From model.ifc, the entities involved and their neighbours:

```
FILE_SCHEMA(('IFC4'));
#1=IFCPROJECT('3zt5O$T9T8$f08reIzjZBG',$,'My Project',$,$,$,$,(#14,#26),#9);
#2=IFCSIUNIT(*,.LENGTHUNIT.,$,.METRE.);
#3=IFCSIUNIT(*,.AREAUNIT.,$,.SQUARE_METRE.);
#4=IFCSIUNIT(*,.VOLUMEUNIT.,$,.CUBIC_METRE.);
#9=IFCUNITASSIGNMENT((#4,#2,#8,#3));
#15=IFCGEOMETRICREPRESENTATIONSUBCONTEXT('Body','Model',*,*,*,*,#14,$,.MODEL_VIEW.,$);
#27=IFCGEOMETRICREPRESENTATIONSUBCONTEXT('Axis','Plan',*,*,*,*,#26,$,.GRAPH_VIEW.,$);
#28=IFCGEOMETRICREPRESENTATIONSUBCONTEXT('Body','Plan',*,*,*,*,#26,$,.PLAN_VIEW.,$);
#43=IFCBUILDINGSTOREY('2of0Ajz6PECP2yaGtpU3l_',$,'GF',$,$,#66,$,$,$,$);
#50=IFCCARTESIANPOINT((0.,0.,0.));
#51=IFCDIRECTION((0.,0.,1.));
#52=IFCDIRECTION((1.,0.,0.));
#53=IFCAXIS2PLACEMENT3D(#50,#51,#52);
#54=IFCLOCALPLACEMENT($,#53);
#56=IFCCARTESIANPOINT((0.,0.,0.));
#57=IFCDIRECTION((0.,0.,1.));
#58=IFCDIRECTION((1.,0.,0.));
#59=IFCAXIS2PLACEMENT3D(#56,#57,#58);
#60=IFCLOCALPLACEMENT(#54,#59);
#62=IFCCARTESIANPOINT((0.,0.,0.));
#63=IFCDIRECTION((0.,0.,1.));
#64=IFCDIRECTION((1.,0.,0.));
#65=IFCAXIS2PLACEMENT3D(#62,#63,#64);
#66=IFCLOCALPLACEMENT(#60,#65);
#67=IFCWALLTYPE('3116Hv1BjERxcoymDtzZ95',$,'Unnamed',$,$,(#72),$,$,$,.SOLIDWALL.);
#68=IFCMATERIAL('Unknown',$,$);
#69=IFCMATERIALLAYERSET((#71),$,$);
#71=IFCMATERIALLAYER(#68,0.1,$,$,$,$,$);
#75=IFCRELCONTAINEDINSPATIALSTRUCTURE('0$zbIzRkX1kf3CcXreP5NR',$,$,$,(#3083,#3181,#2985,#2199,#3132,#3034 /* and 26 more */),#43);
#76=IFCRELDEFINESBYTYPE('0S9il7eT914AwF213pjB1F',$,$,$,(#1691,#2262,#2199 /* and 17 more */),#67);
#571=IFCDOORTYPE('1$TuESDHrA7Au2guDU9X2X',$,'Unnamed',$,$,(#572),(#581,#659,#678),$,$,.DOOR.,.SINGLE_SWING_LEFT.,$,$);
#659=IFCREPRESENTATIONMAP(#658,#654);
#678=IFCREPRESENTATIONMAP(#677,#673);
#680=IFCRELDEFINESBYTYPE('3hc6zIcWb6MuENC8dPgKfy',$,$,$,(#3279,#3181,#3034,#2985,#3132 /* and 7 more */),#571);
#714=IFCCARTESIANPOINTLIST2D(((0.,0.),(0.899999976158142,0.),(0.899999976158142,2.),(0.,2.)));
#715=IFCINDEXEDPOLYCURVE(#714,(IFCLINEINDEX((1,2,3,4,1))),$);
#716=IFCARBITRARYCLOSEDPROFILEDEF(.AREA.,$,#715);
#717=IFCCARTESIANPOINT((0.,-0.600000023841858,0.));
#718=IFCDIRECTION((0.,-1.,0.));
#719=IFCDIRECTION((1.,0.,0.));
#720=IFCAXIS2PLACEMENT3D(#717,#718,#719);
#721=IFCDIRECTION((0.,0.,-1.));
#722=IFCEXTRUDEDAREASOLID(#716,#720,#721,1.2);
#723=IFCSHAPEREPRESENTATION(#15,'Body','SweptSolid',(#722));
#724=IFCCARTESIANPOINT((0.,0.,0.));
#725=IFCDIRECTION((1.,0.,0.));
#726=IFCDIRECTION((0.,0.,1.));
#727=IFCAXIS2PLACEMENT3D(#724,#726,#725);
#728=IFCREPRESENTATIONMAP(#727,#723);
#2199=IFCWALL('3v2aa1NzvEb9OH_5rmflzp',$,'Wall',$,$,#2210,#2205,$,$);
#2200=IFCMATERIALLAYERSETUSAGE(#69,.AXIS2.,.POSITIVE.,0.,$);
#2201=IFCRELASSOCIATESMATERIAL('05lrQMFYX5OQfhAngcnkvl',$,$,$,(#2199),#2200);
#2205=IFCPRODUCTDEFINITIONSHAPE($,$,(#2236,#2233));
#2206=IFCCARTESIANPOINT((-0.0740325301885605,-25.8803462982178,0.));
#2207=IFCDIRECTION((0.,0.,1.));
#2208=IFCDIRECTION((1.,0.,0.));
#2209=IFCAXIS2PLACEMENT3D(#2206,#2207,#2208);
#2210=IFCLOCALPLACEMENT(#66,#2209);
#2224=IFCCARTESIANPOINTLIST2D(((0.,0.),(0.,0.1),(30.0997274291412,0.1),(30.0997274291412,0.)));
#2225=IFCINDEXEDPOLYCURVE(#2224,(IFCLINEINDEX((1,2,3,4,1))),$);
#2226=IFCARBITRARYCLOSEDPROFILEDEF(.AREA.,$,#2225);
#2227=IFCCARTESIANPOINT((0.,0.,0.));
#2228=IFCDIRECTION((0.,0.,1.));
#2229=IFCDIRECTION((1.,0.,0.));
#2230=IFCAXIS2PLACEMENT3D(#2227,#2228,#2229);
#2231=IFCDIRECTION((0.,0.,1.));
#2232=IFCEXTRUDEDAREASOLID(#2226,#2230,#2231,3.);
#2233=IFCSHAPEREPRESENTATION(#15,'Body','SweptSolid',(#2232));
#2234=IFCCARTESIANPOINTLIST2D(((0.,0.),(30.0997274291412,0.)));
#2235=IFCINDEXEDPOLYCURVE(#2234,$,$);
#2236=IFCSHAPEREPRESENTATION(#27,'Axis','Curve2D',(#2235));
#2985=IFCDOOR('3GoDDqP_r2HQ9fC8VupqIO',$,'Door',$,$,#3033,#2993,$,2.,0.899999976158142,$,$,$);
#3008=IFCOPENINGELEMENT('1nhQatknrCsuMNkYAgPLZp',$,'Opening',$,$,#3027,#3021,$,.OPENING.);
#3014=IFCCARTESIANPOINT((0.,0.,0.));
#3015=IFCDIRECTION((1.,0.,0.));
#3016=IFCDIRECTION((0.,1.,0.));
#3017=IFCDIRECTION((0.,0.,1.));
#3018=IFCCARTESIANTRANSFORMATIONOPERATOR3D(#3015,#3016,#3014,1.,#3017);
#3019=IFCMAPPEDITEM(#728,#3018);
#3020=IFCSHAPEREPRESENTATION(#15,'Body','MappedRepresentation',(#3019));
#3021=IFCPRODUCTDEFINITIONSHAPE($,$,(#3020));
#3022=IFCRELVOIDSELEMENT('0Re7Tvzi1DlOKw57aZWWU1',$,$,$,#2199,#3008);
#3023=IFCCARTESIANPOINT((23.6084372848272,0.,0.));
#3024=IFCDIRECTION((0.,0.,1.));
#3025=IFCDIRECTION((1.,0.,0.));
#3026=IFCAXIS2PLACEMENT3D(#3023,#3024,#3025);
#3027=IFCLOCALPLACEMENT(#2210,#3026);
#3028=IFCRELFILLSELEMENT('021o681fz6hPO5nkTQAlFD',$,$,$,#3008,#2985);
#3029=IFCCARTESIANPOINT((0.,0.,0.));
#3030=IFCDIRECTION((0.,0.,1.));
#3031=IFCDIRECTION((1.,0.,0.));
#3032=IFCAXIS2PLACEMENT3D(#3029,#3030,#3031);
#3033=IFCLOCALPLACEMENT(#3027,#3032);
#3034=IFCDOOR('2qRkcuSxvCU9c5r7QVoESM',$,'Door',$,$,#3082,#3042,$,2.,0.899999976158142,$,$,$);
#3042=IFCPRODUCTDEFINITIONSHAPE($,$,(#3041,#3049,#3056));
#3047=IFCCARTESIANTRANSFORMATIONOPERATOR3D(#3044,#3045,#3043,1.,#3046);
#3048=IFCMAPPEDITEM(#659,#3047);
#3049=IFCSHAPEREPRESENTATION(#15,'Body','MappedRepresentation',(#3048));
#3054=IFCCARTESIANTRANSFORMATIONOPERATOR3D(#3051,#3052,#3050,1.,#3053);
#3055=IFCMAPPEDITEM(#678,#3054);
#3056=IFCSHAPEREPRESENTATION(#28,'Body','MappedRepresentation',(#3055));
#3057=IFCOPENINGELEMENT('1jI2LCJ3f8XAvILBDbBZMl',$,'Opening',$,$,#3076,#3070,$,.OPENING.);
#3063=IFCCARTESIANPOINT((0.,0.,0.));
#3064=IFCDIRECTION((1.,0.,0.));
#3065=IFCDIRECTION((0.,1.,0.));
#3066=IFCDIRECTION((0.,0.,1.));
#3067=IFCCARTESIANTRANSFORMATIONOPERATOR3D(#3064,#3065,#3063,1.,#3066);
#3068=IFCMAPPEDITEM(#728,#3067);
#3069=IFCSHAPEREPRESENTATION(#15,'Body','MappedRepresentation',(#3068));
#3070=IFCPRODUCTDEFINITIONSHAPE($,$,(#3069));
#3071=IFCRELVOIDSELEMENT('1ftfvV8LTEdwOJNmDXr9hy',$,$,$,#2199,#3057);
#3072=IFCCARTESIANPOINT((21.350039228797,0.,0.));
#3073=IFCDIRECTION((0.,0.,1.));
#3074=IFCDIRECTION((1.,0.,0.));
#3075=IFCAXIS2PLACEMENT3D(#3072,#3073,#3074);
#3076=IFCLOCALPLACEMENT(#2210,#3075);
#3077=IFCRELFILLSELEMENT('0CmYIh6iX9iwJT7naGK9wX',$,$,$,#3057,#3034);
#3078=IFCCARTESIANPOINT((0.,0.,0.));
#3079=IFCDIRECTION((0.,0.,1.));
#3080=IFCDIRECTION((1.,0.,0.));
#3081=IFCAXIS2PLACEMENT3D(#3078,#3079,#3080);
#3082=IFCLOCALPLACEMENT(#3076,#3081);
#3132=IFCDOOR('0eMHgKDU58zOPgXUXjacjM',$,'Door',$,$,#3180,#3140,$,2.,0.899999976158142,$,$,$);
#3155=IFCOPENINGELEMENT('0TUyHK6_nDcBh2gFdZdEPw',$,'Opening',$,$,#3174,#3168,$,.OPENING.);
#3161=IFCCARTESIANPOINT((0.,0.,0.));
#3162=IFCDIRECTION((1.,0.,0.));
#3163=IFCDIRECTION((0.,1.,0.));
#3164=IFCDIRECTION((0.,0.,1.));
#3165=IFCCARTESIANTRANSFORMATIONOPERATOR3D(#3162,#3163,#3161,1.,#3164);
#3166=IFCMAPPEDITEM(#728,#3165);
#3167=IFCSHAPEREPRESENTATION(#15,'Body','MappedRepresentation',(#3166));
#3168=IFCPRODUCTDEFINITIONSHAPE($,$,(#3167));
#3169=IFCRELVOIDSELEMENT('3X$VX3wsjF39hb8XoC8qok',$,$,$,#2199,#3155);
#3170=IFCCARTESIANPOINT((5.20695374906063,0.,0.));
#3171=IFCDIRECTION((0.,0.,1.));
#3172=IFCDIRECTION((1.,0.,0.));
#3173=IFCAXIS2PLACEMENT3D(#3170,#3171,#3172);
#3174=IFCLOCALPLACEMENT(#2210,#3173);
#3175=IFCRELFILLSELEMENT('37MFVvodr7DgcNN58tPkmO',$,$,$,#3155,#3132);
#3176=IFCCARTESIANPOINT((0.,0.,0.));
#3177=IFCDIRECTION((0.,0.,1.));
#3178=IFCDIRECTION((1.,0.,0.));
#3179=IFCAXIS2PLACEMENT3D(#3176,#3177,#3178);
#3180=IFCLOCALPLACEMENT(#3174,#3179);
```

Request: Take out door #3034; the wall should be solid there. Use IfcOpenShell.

```python
import ifcopenshell
import ifcopenshell.api.feature
import ifcopenshell.api.root
import ifcopenshell.geom
import ifcopenshell.util.shape

model = ifcopenshell.open("model.ifc")
settings = ifcopenshell.geom.settings()


def volume(element):
    """Net volume in cubic metres, openings subtracted."""
    shape = ifcopenshell.geom.create_shape(settings, element)
    return ifcopenshell.util.shape.get_volume(shape.geometry)


door = model.by_guid("2qRkcuSxvCU9c5r7QVoESM")
opening = door.FillsVoids[0].RelatingOpeningElement
wall = opening.VoidsElements[0].RelatingBuildingElement
before = volume(wall)

ifcopenshell.api.root.remove_product(model, product=door)
ifcopenshell.api.feature.remove_feature(model, feature=opening)

after = volume(wall)

print(f"wall volume {before:.3f} -> {after:.3f} m3")

model.write("model_updated.ifc")
```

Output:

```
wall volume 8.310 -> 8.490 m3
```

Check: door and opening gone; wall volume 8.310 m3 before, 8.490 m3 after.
